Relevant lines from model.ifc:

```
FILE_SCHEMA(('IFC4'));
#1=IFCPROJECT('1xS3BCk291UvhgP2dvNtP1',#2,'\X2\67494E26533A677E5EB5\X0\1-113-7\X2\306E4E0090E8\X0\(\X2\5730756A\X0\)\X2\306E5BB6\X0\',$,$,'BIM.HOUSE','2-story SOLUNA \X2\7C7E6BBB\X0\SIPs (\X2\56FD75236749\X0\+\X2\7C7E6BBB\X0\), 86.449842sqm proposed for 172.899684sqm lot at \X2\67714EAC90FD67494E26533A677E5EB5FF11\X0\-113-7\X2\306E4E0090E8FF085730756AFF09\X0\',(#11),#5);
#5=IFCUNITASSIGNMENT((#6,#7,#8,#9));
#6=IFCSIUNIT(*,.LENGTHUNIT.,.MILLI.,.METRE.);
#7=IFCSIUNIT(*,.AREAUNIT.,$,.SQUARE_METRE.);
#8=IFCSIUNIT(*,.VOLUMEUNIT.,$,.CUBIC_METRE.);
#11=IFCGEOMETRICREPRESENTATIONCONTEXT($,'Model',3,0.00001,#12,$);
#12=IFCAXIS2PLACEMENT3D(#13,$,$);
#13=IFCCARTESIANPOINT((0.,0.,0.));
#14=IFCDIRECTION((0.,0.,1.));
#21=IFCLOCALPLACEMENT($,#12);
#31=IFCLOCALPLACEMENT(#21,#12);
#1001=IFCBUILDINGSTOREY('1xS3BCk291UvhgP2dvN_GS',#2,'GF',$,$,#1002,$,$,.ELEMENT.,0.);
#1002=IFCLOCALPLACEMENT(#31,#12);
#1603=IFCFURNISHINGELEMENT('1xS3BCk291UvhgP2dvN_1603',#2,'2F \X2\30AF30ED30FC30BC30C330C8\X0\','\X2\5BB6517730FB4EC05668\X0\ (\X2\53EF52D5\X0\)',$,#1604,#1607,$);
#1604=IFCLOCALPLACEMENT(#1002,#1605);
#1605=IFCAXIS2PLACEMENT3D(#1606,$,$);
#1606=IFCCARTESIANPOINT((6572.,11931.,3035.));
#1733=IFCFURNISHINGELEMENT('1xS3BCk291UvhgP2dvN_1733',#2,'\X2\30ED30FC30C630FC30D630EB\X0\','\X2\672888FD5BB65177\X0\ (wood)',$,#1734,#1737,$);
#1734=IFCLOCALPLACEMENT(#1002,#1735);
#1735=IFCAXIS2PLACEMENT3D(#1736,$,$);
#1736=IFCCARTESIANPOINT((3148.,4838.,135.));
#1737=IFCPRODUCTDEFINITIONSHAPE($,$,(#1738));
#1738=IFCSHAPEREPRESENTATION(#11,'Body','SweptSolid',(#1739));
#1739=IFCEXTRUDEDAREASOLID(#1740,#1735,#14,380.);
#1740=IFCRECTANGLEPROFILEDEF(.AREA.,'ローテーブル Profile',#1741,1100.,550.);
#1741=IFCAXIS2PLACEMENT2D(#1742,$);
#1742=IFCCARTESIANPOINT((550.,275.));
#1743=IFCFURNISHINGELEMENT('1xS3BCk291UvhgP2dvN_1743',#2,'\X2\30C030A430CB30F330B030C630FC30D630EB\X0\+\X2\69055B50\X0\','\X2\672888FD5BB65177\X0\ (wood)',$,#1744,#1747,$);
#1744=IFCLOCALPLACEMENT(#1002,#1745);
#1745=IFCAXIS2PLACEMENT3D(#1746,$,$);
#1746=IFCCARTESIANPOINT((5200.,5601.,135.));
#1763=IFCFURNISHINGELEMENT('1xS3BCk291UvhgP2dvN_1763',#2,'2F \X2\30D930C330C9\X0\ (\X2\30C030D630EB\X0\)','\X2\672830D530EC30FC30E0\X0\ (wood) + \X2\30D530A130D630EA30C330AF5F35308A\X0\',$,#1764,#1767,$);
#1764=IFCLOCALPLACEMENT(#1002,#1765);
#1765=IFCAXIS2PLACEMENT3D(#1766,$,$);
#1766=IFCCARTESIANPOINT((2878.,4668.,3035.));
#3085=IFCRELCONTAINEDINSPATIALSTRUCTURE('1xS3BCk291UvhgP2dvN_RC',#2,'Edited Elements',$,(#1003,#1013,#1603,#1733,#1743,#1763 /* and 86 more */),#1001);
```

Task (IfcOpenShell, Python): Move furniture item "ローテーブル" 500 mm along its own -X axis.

```python
import ifcopenshell
import ifcopenshell.api.geometry
import ifcopenshell.util.placement

model = ifcopenshell.open("model.ifc")

item = model.by_id(1733)
matrix = ifcopenshell.util.placement.get_local_placement(item.ObjectPlacement)
matrix[:3, 3] -= matrix[:3, 0] * 500.0
ifcopenshell.api.geometry.edit_object_placement(model, product=item, matrix=matrix, is_si=False)

print(ifcopenshell.util.placement.get_local_placement(item.ObjectPlacement).round(3) + 0.0)

model.write("model-out.ifc")
```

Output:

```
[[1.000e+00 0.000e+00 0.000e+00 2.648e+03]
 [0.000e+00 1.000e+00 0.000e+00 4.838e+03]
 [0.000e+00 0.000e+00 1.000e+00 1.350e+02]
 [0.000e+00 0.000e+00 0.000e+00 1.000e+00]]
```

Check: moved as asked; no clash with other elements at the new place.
